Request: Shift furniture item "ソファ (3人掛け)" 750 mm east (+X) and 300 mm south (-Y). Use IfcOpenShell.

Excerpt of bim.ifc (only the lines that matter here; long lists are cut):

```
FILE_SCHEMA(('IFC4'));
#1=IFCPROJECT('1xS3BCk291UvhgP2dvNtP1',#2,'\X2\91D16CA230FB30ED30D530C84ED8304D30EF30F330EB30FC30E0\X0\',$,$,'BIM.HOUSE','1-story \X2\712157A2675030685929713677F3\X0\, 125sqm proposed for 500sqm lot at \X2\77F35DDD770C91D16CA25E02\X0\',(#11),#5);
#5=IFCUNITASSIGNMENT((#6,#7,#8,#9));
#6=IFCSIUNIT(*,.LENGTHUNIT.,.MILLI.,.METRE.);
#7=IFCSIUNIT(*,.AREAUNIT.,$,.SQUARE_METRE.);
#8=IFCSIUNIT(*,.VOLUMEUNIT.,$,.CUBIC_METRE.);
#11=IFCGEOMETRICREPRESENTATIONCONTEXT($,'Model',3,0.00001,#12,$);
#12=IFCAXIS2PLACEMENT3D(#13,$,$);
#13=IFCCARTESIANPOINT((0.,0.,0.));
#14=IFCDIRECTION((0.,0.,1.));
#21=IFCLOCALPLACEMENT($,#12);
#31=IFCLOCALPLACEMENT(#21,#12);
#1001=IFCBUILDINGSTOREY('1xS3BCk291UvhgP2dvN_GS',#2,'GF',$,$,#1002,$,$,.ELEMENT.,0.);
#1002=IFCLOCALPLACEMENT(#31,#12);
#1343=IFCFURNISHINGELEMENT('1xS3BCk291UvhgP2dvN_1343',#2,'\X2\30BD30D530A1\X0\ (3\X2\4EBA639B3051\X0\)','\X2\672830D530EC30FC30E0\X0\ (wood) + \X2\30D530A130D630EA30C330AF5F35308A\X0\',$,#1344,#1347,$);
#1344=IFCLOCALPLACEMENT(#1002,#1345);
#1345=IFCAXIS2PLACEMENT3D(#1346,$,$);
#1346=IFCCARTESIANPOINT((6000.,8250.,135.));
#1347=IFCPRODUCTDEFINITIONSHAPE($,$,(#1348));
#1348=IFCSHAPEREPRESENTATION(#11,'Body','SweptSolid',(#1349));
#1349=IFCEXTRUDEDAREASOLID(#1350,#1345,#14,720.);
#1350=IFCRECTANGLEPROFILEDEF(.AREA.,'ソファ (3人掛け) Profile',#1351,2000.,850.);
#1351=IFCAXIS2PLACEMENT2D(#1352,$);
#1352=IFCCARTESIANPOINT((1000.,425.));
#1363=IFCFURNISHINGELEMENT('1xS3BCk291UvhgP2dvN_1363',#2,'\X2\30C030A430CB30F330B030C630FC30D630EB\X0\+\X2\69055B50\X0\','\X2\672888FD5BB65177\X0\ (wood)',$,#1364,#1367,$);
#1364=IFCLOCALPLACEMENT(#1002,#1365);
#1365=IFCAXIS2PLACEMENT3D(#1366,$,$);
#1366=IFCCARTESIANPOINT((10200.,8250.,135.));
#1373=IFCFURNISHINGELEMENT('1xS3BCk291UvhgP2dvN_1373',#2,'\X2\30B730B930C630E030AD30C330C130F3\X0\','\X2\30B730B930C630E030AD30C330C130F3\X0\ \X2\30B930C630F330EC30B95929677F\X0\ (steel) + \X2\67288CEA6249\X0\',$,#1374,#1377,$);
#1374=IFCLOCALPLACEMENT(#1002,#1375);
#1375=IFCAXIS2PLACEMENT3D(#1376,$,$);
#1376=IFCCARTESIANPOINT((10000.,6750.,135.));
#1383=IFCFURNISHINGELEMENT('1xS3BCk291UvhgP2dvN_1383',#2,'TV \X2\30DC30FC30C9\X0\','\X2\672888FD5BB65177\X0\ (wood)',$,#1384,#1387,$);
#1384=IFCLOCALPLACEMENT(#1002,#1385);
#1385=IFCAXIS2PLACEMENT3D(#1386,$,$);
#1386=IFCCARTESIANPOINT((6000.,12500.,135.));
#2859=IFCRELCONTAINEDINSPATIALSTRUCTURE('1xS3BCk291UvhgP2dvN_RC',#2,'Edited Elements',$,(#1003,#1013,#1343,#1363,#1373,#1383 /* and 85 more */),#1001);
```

```python
import ifcopenshell
import ifcopenshell.api.geometry
import ifcopenshell.util.placement
import ifcopenshell.util.unit

model = ifcopenshell.open("bim.ifc")
unit_scale = ifcopenshell.util.unit.calculate_unit_scale(model)

item = model.by_guid("1xS3BCk291UvhgP2dvN_1343")
matrix = ifcopenshell.util.placement.get_local_placement(item.ObjectPlacement)
matrix[0, 3] += 0.75 / unit_scale
matrix[1, 3] -= 0.3 / unit_scale
ifcopenshell.api.geometry.edit_object_placement(model, product=item, matrix=matrix, is_si=False)

print(ifcopenshell.util.placement.get_local_placement(item.ObjectPlacement).round(3) + 0.0)

model.write("bim_rev.ifc")
```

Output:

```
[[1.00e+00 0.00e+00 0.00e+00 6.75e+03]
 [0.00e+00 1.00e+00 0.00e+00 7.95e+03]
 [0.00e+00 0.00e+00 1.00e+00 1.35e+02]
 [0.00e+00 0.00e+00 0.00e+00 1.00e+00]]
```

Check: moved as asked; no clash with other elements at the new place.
